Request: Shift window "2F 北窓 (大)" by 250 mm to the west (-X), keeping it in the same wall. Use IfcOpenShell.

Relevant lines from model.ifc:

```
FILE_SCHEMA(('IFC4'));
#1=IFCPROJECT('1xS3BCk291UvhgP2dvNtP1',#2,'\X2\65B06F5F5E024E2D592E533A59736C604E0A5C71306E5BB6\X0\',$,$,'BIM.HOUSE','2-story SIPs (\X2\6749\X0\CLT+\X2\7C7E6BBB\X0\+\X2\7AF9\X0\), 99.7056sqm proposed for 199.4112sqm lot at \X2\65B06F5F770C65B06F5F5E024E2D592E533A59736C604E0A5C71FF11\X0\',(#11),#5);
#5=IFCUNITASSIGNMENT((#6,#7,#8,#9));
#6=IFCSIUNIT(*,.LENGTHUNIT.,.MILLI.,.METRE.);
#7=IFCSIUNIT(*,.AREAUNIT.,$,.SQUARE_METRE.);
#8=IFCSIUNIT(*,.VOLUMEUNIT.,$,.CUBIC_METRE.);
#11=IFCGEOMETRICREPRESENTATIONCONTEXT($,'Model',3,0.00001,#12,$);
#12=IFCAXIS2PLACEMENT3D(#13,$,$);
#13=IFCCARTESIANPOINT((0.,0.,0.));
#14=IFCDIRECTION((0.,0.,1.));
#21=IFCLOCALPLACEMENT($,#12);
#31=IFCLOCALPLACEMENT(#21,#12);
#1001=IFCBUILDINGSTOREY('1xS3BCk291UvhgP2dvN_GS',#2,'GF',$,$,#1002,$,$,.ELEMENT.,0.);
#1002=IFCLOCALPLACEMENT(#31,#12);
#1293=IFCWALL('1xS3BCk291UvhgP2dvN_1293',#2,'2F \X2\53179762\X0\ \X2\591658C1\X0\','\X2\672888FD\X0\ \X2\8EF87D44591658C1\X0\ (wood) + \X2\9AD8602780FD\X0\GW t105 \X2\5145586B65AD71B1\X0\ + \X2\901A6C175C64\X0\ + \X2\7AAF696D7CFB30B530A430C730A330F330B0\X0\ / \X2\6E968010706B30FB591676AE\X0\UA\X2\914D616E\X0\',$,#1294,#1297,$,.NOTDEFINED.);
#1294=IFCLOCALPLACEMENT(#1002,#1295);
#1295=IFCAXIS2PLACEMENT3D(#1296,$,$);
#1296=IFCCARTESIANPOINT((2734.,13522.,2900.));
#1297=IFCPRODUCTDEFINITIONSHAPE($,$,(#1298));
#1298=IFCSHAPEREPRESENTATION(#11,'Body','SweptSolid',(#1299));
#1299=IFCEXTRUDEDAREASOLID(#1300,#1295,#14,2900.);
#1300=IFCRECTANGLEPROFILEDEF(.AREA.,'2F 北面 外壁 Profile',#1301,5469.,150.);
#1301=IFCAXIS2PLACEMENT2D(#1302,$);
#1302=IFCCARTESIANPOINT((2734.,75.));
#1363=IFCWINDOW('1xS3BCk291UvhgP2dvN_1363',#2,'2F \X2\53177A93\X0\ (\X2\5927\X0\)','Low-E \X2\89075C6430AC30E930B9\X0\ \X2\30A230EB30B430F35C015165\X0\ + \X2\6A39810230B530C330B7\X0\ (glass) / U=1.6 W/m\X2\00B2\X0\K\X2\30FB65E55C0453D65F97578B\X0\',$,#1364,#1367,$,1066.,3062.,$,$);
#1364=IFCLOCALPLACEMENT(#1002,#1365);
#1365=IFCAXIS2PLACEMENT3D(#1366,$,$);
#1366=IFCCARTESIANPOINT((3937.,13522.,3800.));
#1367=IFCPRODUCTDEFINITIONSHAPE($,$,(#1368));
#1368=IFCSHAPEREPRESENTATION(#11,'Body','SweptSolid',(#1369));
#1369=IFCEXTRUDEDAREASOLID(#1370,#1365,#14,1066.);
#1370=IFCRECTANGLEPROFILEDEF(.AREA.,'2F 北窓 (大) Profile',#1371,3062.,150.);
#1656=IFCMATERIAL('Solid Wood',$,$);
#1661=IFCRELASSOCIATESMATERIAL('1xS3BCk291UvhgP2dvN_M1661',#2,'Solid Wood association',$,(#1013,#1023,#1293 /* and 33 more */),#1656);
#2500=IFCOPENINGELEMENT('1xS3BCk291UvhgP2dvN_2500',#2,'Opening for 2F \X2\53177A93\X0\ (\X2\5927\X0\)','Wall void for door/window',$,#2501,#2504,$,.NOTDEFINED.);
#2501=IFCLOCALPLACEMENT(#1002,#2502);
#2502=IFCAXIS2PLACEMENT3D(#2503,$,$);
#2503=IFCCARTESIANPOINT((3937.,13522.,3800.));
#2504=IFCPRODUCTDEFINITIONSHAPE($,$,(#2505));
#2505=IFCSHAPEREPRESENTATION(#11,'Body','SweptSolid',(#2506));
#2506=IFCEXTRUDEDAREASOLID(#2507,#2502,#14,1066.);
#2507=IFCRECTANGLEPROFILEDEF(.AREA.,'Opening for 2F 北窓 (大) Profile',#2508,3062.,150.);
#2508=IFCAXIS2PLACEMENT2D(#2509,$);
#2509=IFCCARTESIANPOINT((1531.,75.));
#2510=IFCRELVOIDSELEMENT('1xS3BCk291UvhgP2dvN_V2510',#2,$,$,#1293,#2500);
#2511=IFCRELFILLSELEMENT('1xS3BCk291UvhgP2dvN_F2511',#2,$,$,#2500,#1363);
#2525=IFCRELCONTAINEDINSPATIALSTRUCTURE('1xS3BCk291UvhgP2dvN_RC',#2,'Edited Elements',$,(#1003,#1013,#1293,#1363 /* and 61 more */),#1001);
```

```python
import ifcopenshell
import ifcopenshell.api.geometry
import ifcopenshell.util.placement

model = ifcopenshell.open("model.ifc")

window = model.by_guid("1xS3BCk291UvhgP2dvN_1363")
opening = window.FillsVoids[0].RelatingOpeningElement
wall = opening.VoidsElements[0].RelatingBuildingElement

wall_matrix = ifcopenshell.util.placement.get_local_placement(wall.ObjectPlacement)
shift = wall_matrix[:3, 0] * -250.0
before = ifcopenshell.util.placement.get_local_placement(window.ObjectPlacement)[:3, 3].copy()

# The window is not placed relative to its opening, so move both.
for product in (opening, window):
    matrix = ifcopenshell.util.placement.get_local_placement(product.ObjectPlacement)
    matrix[:3, 3] += shift
    ifcopenshell.api.geometry.edit_object_placement(model, product=product, matrix=matrix, is_si=False)

after = ifcopenshell.util.placement.get_local_placement(window.ObjectPlacement)[:3, 3]
print("window moved by", (after - before).round(3) + 0.0)

model.write("model_rev.ifc")
```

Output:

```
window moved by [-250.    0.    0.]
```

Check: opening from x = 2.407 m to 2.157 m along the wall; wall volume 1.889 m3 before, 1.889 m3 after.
